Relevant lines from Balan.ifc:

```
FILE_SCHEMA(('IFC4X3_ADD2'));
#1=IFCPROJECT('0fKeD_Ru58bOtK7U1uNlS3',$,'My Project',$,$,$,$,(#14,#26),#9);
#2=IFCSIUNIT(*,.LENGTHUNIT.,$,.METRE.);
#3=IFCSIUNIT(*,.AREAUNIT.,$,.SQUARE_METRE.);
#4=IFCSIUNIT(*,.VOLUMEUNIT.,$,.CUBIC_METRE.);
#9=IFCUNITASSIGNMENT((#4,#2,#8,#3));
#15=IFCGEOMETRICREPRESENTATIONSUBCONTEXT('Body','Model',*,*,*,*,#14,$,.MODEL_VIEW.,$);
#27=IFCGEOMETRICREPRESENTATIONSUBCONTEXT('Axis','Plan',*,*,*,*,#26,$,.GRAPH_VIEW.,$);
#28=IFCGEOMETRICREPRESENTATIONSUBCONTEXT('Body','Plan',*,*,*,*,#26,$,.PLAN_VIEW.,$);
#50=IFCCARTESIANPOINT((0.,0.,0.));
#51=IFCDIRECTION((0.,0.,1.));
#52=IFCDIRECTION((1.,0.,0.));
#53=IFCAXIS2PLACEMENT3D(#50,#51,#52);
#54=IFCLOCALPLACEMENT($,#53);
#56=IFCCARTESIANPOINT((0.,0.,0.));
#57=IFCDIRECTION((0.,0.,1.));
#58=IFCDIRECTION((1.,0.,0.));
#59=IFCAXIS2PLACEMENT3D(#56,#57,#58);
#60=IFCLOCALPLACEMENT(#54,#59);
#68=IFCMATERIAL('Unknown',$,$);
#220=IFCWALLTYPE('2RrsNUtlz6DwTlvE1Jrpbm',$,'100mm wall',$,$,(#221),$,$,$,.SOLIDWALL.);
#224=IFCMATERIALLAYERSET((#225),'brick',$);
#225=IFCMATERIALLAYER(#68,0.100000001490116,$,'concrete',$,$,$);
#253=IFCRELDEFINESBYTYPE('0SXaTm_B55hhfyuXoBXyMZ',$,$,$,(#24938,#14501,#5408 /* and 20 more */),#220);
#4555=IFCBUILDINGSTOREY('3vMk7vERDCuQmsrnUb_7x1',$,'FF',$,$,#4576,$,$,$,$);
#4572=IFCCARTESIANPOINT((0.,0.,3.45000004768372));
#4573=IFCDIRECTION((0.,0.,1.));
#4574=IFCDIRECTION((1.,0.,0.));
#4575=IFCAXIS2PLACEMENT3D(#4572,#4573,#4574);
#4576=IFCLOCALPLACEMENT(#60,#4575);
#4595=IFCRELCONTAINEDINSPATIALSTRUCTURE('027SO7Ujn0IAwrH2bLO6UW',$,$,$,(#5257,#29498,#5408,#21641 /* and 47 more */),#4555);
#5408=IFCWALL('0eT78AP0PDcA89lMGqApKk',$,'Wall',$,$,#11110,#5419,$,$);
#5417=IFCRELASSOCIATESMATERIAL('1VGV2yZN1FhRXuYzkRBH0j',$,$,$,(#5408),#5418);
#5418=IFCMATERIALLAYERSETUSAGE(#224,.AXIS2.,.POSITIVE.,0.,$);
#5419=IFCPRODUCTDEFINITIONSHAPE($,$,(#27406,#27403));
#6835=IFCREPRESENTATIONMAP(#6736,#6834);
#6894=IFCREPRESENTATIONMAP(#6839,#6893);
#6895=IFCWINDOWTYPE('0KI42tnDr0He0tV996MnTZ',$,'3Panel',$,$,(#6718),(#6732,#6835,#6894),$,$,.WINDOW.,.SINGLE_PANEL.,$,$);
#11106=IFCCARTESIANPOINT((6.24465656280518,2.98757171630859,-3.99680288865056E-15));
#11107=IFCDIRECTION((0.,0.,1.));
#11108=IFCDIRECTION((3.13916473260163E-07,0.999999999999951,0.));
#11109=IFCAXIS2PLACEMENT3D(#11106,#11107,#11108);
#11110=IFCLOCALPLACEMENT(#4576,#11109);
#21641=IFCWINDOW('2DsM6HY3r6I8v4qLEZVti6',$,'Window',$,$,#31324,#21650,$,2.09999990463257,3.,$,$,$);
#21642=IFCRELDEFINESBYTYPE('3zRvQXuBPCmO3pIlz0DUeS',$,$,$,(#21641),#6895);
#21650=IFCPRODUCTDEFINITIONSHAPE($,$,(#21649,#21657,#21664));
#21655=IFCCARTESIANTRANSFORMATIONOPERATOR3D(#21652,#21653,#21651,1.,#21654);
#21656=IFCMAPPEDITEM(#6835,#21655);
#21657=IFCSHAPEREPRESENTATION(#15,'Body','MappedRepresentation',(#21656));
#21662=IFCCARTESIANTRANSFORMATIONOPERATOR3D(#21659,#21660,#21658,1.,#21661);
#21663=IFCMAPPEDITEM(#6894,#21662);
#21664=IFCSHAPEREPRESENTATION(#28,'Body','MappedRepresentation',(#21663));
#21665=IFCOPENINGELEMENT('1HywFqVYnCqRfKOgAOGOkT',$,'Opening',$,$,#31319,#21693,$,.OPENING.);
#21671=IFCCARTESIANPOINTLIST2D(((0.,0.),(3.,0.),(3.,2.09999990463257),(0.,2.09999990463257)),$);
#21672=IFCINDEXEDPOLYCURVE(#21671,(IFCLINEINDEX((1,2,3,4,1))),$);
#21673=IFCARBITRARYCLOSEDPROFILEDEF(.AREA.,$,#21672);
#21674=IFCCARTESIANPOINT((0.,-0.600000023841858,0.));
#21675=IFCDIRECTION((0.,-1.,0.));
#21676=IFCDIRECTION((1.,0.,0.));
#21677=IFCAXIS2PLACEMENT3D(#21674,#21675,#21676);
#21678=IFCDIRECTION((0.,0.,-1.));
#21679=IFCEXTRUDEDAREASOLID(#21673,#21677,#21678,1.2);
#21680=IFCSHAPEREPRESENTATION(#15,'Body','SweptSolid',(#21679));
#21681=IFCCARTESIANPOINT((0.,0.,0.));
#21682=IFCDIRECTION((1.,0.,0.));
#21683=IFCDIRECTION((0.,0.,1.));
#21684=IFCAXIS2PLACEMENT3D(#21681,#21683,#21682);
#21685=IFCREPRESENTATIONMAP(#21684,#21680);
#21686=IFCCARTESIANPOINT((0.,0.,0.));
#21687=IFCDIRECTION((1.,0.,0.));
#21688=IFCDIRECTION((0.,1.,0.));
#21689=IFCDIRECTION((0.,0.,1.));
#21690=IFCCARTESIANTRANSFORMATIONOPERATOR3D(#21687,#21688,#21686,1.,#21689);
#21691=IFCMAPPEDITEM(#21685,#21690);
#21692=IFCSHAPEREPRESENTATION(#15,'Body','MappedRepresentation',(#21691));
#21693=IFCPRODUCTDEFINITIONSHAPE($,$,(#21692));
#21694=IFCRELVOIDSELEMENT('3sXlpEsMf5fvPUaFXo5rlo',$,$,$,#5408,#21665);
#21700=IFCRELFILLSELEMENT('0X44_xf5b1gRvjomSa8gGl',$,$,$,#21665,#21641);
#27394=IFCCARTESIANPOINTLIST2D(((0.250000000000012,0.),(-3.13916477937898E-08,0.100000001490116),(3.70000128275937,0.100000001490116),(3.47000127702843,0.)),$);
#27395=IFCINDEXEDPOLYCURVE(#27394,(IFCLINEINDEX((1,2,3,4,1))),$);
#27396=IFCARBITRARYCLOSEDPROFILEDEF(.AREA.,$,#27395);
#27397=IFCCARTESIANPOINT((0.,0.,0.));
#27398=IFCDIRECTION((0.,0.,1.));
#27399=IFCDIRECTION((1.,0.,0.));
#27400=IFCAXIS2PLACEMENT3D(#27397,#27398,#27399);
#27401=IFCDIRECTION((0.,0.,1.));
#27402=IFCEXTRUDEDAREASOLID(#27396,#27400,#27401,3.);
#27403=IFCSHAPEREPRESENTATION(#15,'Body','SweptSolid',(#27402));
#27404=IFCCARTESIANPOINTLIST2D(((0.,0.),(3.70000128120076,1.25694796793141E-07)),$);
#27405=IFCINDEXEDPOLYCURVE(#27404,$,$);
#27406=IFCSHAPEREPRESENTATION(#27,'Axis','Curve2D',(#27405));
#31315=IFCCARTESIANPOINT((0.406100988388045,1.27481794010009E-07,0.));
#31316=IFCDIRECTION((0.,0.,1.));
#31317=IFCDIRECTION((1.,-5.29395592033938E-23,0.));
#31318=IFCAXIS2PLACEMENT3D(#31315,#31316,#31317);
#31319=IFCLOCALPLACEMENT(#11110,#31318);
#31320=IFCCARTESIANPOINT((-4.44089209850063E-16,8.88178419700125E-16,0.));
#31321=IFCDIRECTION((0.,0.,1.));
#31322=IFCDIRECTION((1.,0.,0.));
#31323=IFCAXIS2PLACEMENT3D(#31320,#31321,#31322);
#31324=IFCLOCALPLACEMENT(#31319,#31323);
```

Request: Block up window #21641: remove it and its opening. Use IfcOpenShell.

```python
import ifcopenshell
import ifcopenshell.api.feature
import ifcopenshell.api.root
import ifcopenshell.geom
import ifcopenshell.util.shape

model = ifcopenshell.open("Balan.ifc")
settings = ifcopenshell.geom.settings()


def volume(element):
    """Net volume in cubic metres, openings subtracted."""
    shape = ifcopenshell.geom.create_shape(settings, element)
    return ifcopenshell.util.shape.get_volume(shape.geometry)


window = model.by_guid("2DsM6HY3r6I8v4qLEZVti6")
opening = window.FillsVoids[0].RelatingOpeningElement
wall = opening.VoidsElements[0].RelatingBuildingElement
before = volume(wall)

ifcopenshell.api.root.remove_product(model, product=window)
ifcopenshell.api.feature.remove_feature(model, feature=opening)

after = volume(wall)

print(f"wall volume {before:.3f} -> {after:.3f} m3")

model.write("Balan-out.ifc")
```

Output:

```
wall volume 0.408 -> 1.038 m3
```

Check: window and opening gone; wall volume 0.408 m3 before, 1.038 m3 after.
